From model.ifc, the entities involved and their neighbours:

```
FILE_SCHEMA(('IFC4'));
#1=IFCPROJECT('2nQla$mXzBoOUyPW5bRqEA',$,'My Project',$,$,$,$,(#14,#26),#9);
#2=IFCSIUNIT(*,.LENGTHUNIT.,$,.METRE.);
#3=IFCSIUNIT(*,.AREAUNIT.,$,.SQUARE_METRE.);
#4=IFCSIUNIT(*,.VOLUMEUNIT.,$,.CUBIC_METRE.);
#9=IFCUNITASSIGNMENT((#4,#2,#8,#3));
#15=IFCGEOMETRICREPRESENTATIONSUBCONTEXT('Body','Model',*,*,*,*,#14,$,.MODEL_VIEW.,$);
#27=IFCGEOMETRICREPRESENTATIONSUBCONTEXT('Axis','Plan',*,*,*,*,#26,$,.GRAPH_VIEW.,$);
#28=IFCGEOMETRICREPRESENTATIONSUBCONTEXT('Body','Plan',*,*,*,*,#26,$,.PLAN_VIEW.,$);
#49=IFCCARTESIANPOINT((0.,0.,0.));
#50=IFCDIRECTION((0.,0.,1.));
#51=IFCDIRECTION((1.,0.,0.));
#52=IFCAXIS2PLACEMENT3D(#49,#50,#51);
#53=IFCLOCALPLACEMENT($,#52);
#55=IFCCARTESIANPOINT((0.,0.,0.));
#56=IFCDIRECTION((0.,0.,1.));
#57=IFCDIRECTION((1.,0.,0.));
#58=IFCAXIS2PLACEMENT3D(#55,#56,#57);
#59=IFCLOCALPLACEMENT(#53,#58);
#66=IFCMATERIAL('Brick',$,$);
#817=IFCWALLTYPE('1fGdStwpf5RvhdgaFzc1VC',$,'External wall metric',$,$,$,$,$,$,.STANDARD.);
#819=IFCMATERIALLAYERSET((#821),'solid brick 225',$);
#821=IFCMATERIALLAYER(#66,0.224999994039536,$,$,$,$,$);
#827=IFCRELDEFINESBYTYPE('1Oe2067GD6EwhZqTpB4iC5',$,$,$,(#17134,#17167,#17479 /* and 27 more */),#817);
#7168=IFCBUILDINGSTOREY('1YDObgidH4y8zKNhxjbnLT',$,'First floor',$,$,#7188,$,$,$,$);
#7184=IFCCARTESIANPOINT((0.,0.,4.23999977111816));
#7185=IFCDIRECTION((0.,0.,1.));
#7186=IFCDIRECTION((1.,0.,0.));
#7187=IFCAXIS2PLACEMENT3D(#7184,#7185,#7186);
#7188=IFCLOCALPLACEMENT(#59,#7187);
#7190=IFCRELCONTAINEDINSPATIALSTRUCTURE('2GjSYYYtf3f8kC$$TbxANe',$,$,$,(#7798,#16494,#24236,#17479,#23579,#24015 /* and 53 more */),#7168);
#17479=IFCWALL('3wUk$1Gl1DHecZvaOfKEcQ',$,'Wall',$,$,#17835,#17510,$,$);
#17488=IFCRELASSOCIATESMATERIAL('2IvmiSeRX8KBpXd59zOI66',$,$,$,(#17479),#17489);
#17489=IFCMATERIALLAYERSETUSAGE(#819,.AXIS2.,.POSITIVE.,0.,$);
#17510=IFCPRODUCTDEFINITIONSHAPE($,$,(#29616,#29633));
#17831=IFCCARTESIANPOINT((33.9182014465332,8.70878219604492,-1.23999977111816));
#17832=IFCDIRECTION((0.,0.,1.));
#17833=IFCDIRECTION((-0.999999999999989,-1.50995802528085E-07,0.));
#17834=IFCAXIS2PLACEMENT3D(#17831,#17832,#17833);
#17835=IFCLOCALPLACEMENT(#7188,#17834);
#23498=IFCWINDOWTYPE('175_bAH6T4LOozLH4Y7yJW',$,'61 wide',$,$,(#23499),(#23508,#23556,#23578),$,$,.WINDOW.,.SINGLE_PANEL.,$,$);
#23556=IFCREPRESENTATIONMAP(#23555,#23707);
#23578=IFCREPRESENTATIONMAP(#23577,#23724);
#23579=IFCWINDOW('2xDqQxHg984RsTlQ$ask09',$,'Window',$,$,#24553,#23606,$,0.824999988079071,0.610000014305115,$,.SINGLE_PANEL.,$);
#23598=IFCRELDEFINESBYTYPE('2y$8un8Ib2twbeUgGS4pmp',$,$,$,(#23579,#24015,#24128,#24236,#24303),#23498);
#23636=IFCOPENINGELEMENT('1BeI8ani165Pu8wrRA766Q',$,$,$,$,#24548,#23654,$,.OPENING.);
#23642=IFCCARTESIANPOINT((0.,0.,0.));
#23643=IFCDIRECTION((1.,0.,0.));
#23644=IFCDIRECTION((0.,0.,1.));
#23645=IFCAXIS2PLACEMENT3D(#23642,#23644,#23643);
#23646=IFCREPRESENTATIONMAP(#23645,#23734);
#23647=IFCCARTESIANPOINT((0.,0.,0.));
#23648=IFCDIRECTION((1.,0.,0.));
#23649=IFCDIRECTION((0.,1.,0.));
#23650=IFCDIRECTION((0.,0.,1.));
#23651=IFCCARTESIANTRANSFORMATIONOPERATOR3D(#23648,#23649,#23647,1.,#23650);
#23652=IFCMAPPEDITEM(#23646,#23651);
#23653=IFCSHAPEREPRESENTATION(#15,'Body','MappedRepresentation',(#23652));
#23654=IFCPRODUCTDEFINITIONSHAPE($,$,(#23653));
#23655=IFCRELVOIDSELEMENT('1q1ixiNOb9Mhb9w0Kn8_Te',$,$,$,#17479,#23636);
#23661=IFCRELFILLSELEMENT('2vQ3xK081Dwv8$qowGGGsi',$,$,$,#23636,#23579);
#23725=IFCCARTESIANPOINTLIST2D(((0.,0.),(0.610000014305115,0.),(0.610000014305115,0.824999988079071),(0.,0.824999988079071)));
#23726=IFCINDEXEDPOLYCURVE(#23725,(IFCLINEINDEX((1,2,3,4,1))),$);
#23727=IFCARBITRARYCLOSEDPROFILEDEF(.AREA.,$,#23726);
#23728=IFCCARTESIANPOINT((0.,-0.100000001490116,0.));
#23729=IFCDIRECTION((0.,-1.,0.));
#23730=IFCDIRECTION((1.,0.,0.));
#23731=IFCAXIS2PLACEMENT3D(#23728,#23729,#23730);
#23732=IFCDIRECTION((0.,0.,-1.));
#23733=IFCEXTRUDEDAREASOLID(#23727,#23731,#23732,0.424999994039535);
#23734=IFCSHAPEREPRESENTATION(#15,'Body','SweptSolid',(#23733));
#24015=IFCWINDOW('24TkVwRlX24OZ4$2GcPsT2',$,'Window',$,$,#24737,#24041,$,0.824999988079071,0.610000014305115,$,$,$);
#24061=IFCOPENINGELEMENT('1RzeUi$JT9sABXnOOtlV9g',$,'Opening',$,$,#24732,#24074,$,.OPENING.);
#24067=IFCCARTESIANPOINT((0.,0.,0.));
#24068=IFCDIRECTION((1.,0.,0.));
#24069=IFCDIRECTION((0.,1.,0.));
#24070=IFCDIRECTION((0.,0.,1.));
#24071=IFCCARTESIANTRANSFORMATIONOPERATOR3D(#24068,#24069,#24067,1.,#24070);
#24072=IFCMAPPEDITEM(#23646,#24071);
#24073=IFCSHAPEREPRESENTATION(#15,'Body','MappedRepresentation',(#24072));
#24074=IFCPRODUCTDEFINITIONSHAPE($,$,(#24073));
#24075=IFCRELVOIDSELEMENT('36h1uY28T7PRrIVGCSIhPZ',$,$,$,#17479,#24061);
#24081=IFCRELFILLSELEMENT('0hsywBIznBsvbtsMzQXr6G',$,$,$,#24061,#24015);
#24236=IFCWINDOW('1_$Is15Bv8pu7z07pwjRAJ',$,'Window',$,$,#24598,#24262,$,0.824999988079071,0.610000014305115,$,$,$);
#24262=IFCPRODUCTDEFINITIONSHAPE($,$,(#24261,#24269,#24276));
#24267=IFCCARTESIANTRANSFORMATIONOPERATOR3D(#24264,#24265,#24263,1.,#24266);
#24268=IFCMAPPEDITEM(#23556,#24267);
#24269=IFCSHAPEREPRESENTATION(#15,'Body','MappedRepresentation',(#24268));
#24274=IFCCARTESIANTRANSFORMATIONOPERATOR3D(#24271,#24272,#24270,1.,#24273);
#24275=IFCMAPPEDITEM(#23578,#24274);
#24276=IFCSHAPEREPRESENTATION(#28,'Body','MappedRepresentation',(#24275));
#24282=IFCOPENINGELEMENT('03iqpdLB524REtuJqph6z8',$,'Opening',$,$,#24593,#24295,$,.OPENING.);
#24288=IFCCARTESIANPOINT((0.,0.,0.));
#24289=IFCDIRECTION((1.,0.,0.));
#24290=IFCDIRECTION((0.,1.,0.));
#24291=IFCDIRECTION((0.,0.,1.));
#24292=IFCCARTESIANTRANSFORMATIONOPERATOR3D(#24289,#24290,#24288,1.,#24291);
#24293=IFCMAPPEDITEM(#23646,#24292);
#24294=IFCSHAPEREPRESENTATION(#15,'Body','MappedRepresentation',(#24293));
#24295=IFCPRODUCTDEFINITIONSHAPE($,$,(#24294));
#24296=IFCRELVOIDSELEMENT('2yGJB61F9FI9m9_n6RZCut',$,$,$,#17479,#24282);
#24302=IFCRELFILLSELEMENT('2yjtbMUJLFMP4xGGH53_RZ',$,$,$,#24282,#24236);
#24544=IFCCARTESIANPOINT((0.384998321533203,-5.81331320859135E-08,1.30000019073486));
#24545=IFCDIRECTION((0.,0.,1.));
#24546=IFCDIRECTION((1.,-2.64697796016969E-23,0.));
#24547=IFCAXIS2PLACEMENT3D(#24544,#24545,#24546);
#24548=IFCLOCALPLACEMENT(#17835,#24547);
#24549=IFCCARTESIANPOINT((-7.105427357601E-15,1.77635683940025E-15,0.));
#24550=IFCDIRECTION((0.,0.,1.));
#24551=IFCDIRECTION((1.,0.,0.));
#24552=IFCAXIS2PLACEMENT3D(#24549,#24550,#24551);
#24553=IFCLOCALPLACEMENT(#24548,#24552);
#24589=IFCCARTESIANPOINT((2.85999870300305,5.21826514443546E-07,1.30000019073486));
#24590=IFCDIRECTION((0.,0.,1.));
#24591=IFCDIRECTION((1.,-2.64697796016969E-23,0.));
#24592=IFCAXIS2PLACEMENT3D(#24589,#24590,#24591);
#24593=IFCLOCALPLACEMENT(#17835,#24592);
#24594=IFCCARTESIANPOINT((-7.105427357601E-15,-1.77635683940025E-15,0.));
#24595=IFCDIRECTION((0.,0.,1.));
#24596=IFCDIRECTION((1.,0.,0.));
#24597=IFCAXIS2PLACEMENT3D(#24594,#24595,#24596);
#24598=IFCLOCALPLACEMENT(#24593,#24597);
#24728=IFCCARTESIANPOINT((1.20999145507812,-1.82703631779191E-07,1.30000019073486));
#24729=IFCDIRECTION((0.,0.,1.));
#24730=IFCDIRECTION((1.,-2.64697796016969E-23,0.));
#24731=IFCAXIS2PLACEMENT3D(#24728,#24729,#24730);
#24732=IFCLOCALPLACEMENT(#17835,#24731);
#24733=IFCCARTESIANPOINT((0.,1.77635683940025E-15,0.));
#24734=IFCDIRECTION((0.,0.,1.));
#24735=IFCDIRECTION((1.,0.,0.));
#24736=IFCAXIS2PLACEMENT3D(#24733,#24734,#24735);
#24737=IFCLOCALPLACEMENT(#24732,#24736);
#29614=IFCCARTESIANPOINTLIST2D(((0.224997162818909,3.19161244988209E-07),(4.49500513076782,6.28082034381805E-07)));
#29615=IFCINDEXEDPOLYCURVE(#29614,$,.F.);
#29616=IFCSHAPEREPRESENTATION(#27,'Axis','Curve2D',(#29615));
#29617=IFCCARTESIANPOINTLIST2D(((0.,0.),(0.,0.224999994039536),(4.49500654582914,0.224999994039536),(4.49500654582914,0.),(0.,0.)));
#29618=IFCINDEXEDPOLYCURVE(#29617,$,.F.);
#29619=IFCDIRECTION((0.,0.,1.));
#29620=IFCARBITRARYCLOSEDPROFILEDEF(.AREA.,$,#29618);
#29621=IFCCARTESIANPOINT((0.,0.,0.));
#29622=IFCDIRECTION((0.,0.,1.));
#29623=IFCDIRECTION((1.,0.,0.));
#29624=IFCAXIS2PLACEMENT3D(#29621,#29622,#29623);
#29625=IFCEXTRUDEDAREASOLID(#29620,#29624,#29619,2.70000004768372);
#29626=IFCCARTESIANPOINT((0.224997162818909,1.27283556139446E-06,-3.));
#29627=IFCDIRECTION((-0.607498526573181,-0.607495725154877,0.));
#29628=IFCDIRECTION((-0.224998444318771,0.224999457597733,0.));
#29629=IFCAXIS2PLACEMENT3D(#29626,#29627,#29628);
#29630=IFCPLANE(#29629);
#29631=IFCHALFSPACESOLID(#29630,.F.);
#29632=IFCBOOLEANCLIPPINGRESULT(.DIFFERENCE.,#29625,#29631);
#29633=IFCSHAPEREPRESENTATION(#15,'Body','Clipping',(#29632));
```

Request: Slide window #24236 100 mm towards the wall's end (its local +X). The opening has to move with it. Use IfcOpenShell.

```python
import ifcopenshell
import ifcopenshell.api.geometry
import ifcopenshell.util.placement

model = ifcopenshell.open("model.ifc")

window = model.by_guid("1_$Is15Bv8pu7z07pwjRAJ")
opening = window.FillsVoids[0].RelatingOpeningElement
wall = opening.VoidsElements[0].RelatingBuildingElement

wall_matrix = ifcopenshell.util.placement.get_local_placement(wall.ObjectPlacement)
shift = wall_matrix[:3, 0] * 0.1
before = ifcopenshell.util.placement.get_local_placement(window.ObjectPlacement)[:3, 3].copy()

# The window is placed relative to its opening, so it follows when the opening moves.
matrix = ifcopenshell.util.placement.get_local_placement(opening.ObjectPlacement)
matrix[:3, 3] += shift
ifcopenshell.api.geometry.edit_object_placement(
    model, product=opening, matrix=matrix, is_si=False, should_transform_children=True
)

after = ifcopenshell.util.placement.get_local_placement(window.ObjectPlacement)[:3, 3]
print("window moved by", (after - before).round(3) + 0.0)

model.write("model_edited.ifc")
```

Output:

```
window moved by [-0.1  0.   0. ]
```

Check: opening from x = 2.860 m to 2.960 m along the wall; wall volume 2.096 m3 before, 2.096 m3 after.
